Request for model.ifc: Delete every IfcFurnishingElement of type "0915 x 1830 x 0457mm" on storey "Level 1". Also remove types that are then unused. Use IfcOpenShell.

First a look at what the model holds.

```python
import ifcopenshell
import ifcopenshell.util.element

model = ifcopenshell.open("model.ifc")
print(model.schema)
storey = next(s for s in model.by_type("IfcBuildingStorey") if s.Name == "Level 1")
furniture = [e for e in ifcopenshell.util.element.get_decomposition(storey) if e.is_a("IfcFurnishingElement")]
seen = {}
for e in furniture:
    element_type = ifcopenshell.util.element.get_type(e)
    name = element_type.Name if element_type not in (None, e) else None
    seen[name] = seen.get(name, 0) + 1
for name, count in sorted(seen.items(), key=str):
    print(count, "x", name)
```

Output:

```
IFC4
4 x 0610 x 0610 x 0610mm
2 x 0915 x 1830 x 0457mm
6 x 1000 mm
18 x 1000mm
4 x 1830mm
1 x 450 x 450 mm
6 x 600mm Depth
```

```python
import ifcopenshell
import ifcopenshell.api.root
import ifcopenshell.util.element

model = ifcopenshell.open("model.ifc")

storey = next(s for s in model.by_type("IfcBuildingStorey") if s.Name == "Level 1")
furniture = [e for e in ifcopenshell.util.element.get_decomposition(storey) if e.is_a("IfcFurnishingElement")]
targets = [e for e in furniture if (t := ifcopenshell.util.element.get_type(e)) not in (None, e) and t.Name == "0915 x 1830 x 0457mm"]
types = {ifcopenshell.util.element.get_type(e) for e in targets} - {None, *targets}

for e in targets:
    ifcopenshell.api.root.remove_product(model, product=e)
print(len(targets), "removed")

unused = [t for t in types if not ifcopenshell.util.element.get_types(t)]
for t in unused:
    ifcopenshell.api.root.remove_product(model, product=t)
print(len(unused), "unused types removed")

model.write("model_rev.ifc")
```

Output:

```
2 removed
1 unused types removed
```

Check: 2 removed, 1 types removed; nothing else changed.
